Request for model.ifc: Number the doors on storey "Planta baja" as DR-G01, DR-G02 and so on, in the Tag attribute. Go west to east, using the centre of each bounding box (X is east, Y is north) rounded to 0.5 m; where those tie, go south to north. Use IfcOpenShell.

First a look at what the model holds.

```python
import ifcopenshell
import ifcopenshell.util.element
import ifcopenshell.util.placement

model = ifcopenshell.open("model.ifc")
print(model.schema)
storey = next(s for s in model.by_type("IfcBuildingStorey") if s.Name == "Planta baja")
doors = [e for e in ifcopenshell.util.element.get_decomposition(storey) if e.is_a("IfcDoor")]
for e in sorted(doors, key=lambda e: e.id()):
    origin = ifcopenshell.util.placement.get_local_placement(e.ObjectPlacement)[:3, 3]
    print(e.id(), e.Tag, e.Name, origin.round(2) + 0.0, sep=" | ")
```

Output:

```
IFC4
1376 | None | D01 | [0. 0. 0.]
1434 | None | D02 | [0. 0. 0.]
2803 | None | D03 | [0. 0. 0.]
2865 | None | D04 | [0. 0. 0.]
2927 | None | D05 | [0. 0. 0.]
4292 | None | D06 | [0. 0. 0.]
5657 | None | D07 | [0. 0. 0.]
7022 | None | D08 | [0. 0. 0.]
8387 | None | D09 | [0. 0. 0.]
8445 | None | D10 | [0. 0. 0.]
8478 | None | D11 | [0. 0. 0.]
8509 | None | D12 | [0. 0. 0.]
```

```python
import ifcopenshell
import ifcopenshell.geom
import ifcopenshell.util.element
import ifcopenshell.util.shape

model = ifcopenshell.open("model.ifc")
settings = ifcopenshell.geom.settings()
settings.set("use-world-coords", True)


def centre(element):
    shape = ifcopenshell.geom.create_shape(settings, element)
    return ifcopenshell.util.shape.get_bbox_centroid(shape.geometry)


storey = next(s for s in model.by_type("IfcBuildingStorey") if s.Name == "Planta baja")
doors = [e for e in ifcopenshell.util.element.get_decomposition(storey) if e.is_a("IfcDoor")]

# Insertion points can sit at a corner or the storey origin, so sort by the geometry (in metres).
centres = {e: centre(e) for e in doors}
doors.sort(key=lambda e: (round(centres[e][0] / 0.5), centres[e][1]))

for i, e in enumerate(doors, start=1):
    number = f"DR-G{i:02d}"
    e.Tag = number
    print(e.id(), number)

model.write("model_rev.ifc")
```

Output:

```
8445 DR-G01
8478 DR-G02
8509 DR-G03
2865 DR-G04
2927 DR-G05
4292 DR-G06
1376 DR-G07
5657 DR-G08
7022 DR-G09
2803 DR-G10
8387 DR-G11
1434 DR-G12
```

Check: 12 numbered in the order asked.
